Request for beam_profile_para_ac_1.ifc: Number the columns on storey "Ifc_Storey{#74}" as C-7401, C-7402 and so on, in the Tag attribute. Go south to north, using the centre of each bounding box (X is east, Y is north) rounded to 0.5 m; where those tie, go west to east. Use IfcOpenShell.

First a look at what the model holds.

```python
import ifcopenshell
import ifcopenshell.util.element
import ifcopenshell.util.placement

model = ifcopenshell.open("beam_profile_para_ac_1.ifc")
print(model.schema)
storey = next(s for s in model.by_type("IfcBuildingStorey") if s.Name == "Ifc_Storey{#74}")
columns = [e for e in ifcopenshell.util.element.get_decomposition(storey) if e.is_a("IfcColumn")]
for e in sorted(columns, key=lambda e: e.id()):
    origin = ifcopenshell.util.placement.get_local_placement(e.ObjectPlacement)[:3, 3]
    print(e.id(), e.Tag, e.Name, origin.round(2) + 0.0, sep=" | ")
```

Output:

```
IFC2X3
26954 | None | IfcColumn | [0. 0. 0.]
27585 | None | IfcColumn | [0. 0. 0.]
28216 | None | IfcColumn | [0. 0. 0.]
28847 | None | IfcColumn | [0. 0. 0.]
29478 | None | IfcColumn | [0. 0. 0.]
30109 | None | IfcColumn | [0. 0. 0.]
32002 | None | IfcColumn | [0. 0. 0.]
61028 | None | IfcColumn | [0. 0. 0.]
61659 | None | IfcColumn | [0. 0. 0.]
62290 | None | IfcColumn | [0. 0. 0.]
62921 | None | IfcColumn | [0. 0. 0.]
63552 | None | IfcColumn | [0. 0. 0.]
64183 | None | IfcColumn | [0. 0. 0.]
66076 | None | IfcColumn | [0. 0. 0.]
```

```python
import ifcopenshell
import ifcopenshell.geom
import ifcopenshell.util.element
import ifcopenshell.util.shape

model = ifcopenshell.open("beam_profile_para_ac_1.ifc")
settings = ifcopenshell.geom.settings()
settings.set("use-world-coords", True)


def centre(element):
    shape = ifcopenshell.geom.create_shape(settings, element)
    return ifcopenshell.util.shape.get_bbox_centroid(shape.geometry)


storey = next(s for s in model.by_type("IfcBuildingStorey") if s.Name == "Ifc_Storey{#74}")
columns = [e for e in ifcopenshell.util.element.get_decomposition(storey) if e.is_a("IfcColumn")]

# Insertion points can sit at a corner or the storey origin, so sort by the geometry (in metres).
centres = {e: centre(e) for e in columns}
columns.sort(key=lambda e: (round(centres[e][1] / 0.5), centres[e][0]))

for i, e in enumerate(columns, start=1):
    number = f"C-74{i:02d}"
    e.Tag = number
    print(e.id(), number)

model.write("beam_profile_para_ac_1_v2.ifc")
```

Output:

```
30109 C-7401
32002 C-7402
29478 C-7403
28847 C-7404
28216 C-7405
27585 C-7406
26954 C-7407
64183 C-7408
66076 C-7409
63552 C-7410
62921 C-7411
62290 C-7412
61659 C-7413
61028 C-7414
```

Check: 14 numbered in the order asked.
